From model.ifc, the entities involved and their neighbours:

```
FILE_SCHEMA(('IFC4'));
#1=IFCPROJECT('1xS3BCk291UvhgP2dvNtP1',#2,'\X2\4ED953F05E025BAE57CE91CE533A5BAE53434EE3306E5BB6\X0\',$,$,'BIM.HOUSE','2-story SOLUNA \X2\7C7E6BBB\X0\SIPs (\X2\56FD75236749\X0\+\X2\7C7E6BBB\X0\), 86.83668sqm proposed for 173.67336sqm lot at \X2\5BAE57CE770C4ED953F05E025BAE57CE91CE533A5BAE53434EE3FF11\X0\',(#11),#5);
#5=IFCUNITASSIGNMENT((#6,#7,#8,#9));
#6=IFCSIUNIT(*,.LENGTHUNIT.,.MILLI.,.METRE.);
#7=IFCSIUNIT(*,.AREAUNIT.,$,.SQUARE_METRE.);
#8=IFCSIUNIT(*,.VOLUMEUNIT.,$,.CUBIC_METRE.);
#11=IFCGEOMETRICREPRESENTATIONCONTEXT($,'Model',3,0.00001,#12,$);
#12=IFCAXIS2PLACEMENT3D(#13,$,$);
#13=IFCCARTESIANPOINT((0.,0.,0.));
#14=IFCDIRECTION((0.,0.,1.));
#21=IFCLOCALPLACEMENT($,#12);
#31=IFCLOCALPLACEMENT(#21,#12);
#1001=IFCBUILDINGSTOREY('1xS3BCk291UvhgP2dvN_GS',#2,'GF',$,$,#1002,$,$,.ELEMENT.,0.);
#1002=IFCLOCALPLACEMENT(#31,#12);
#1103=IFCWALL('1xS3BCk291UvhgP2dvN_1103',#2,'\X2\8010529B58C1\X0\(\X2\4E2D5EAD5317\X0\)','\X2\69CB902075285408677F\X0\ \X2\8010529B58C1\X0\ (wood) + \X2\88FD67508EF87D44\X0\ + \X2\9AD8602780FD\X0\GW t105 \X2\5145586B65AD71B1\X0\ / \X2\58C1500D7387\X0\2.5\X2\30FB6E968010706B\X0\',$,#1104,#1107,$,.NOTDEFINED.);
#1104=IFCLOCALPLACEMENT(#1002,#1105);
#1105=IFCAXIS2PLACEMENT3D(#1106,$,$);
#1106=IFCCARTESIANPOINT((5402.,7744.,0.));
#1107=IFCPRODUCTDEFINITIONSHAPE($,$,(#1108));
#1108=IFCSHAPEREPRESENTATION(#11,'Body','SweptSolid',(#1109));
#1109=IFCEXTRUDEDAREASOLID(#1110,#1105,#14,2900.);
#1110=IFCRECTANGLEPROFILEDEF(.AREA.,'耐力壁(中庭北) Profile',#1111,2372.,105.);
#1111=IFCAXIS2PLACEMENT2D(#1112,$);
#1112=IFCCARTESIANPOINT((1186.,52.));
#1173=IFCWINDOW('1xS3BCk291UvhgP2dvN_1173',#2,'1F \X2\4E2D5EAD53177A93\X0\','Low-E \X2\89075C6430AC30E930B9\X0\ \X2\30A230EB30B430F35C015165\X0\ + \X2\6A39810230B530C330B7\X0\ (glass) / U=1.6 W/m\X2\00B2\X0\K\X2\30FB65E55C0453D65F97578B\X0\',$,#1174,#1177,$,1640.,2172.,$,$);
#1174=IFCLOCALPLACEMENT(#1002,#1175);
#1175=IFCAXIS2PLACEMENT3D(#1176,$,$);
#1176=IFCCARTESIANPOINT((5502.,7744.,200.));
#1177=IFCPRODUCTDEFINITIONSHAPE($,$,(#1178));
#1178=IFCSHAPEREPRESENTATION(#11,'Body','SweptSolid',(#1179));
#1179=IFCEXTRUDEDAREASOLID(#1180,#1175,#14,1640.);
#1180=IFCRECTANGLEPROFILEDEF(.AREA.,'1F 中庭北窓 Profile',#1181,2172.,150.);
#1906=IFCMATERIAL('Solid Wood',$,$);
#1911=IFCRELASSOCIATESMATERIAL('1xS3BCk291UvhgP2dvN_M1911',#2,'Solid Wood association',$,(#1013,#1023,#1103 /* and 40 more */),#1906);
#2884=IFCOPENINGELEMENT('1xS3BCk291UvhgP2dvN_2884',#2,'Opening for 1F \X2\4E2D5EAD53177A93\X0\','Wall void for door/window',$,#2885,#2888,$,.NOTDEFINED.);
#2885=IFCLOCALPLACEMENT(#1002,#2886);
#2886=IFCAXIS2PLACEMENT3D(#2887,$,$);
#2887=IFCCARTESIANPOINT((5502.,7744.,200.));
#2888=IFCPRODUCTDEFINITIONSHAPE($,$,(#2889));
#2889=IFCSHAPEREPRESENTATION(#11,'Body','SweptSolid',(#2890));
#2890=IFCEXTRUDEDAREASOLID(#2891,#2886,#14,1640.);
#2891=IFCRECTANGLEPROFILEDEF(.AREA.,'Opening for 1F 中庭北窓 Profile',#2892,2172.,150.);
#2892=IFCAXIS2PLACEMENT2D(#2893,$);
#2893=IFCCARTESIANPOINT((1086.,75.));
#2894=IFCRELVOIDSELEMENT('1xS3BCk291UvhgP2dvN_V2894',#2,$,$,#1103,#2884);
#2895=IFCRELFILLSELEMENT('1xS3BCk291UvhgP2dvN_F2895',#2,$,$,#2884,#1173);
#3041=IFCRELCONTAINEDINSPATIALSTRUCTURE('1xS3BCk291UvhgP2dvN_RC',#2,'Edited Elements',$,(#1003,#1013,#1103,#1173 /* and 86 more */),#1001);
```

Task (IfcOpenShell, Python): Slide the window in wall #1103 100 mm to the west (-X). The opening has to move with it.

```python
import ifcopenshell
import ifcopenshell.api.geometry
import ifcopenshell.util.placement
import ifcopenshell.util.unit

model = ifcopenshell.open("model.ifc")
unit_scale = ifcopenshell.util.unit.calculate_unit_scale(model)

window = model.by_id(1173)
opening = window.FillsVoids[0].RelatingOpeningElement
wall = opening.VoidsElements[0].RelatingBuildingElement

wall_matrix = ifcopenshell.util.placement.get_local_placement(wall.ObjectPlacement)
shift = wall_matrix[:3, 0] * -0.1 / unit_scale
before = ifcopenshell.util.placement.get_local_placement(window.ObjectPlacement)[:3, 3].copy()

# The window is not placed relative to its opening, so move both.
for product in (opening, window):
    matrix = ifcopenshell.util.placement.get_local_placement(product.ObjectPlacement)
    matrix[:3, 3] += shift
    ifcopenshell.api.geometry.edit_object_placement(model, product=product, matrix=matrix, is_si=False)

after = ifcopenshell.util.placement.get_local_placement(window.ObjectPlacement)[:3, 3]
print("window moved by", (after - before).round(3) + 0.0)

model.write("model_v2.ifc")
```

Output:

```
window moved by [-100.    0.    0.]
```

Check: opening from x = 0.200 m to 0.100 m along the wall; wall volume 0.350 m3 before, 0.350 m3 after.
